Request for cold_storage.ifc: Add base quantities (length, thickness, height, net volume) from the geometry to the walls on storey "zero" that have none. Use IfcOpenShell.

First a look at what the model holds.

```python
import ifcopenshell
import ifcopenshell.util.element
import ifcopenshell.util.unit

model = ifcopenshell.open("cold_storage.ifc")
print(model.schema)
for unit_type in ("LENGTHUNIT", "AREAUNIT", "VOLUMEUNIT"):
    print(unit_type, ifcopenshell.util.unit.calculate_unit_scale(model, unit_type))
storey = next(s for s in model.by_type("IfcBuildingStorey") if s.Name == "zero")
walls = [e for e in ifcopenshell.util.element.get_decomposition(storey) if e.is_a("IfcWall")]
for e in sorted(walls, key=lambda e: e.id()):
    print(e.id(), e.is_a(), e.Name, list(ifcopenshell.util.element.get_psets(e, qtos_only=True)), sep=" | ")
```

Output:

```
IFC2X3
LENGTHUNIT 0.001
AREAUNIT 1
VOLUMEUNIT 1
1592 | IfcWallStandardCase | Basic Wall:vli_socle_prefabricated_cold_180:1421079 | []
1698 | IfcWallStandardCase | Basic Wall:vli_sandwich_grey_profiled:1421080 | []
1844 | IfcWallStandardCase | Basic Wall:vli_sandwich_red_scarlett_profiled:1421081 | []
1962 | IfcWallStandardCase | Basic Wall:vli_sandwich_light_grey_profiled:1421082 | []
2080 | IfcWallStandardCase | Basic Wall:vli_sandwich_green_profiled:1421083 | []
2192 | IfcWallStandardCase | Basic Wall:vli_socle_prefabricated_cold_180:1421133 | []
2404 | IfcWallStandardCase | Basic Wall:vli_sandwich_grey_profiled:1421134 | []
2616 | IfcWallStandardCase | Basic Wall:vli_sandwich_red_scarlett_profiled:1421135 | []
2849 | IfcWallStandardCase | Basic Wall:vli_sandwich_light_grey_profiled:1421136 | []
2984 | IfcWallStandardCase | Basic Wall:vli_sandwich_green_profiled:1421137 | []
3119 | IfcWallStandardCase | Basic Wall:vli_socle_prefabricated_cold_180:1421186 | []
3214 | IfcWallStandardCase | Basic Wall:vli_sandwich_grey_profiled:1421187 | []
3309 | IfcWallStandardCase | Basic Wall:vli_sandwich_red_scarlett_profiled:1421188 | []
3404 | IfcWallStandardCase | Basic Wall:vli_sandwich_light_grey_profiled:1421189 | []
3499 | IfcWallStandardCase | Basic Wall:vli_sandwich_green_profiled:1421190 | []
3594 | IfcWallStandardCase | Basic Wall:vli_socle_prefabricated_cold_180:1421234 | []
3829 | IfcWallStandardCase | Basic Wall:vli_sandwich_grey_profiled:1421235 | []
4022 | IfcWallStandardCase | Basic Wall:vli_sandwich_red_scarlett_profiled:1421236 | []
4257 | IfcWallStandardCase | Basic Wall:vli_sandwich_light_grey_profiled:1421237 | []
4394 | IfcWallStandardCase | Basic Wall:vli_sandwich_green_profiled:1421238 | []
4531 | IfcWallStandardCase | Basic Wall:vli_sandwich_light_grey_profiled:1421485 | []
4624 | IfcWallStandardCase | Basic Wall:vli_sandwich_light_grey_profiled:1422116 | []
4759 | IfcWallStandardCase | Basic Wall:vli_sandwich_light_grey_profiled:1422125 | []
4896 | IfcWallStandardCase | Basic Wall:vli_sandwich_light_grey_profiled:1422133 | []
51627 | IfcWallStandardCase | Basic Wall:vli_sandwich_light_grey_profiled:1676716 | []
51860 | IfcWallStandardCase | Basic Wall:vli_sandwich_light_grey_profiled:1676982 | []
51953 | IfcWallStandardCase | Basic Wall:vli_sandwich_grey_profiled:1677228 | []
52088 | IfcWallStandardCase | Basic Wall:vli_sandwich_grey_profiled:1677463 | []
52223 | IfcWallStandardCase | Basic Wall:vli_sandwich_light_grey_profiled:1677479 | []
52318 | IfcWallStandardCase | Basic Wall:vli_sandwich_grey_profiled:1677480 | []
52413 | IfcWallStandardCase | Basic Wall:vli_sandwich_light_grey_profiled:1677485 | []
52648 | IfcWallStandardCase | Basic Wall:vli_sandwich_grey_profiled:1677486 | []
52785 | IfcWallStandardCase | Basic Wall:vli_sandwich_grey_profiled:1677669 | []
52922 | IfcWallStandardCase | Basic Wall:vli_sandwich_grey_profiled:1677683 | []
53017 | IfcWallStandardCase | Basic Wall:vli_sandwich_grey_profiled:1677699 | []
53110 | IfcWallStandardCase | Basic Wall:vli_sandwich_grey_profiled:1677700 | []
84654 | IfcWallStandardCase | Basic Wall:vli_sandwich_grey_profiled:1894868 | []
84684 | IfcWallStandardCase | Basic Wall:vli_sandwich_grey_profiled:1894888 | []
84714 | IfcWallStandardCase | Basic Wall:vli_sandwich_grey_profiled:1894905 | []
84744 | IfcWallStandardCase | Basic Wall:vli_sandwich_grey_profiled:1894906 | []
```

```python
import ifcopenshell
import ifcopenshell.api.pset
import ifcopenshell.geom
import ifcopenshell.util.element
import ifcopenshell.util.shape
import ifcopenshell.util.unit

model = ifcopenshell.open("cold_storage.ifc")
unit_scale = ifcopenshell.util.unit.calculate_unit_scale(model)
volume_scale = ifcopenshell.util.unit.calculate_unit_scale(model, "VOLUMEUNIT")
settings = ifcopenshell.geom.settings()

storey = next(s for s in model.by_type("IfcBuildingStorey") if s.Name == "zero")
walls = [e for e in ifcopenshell.util.element.get_decomposition(storey) if e.is_a("IfcWall")]

for e in sorted(walls, key=lambda e: e.id()):
    if ifcopenshell.util.element.get_psets(e, qtos_only=True, should_inherit=False):
        continue
    # Geometry comes back in metres, in the element's own axes.
    shape = ifcopenshell.geom.create_shape(settings, e)
    values = {
        "Length": ifcopenshell.util.shape.get_x(shape.geometry) / unit_scale,
        "Width": ifcopenshell.util.shape.get_y(shape.geometry) / unit_scale,
        "Height": ifcopenshell.util.shape.get_z(shape.geometry) / unit_scale,
        "NetVolume": ifcopenshell.util.shape.get_volume(shape.geometry) / volume_scale,
    }
    qto = ifcopenshell.api.pset.add_qto(model, product=e, name="BaseQuantities")
    ifcopenshell.api.pset.edit_qto(model, qto=qto, properties=values)
    print(e.id(), {k: round(v, 3) for k, v in values.items()})

model.write("cold_storage_v2.ifc")
```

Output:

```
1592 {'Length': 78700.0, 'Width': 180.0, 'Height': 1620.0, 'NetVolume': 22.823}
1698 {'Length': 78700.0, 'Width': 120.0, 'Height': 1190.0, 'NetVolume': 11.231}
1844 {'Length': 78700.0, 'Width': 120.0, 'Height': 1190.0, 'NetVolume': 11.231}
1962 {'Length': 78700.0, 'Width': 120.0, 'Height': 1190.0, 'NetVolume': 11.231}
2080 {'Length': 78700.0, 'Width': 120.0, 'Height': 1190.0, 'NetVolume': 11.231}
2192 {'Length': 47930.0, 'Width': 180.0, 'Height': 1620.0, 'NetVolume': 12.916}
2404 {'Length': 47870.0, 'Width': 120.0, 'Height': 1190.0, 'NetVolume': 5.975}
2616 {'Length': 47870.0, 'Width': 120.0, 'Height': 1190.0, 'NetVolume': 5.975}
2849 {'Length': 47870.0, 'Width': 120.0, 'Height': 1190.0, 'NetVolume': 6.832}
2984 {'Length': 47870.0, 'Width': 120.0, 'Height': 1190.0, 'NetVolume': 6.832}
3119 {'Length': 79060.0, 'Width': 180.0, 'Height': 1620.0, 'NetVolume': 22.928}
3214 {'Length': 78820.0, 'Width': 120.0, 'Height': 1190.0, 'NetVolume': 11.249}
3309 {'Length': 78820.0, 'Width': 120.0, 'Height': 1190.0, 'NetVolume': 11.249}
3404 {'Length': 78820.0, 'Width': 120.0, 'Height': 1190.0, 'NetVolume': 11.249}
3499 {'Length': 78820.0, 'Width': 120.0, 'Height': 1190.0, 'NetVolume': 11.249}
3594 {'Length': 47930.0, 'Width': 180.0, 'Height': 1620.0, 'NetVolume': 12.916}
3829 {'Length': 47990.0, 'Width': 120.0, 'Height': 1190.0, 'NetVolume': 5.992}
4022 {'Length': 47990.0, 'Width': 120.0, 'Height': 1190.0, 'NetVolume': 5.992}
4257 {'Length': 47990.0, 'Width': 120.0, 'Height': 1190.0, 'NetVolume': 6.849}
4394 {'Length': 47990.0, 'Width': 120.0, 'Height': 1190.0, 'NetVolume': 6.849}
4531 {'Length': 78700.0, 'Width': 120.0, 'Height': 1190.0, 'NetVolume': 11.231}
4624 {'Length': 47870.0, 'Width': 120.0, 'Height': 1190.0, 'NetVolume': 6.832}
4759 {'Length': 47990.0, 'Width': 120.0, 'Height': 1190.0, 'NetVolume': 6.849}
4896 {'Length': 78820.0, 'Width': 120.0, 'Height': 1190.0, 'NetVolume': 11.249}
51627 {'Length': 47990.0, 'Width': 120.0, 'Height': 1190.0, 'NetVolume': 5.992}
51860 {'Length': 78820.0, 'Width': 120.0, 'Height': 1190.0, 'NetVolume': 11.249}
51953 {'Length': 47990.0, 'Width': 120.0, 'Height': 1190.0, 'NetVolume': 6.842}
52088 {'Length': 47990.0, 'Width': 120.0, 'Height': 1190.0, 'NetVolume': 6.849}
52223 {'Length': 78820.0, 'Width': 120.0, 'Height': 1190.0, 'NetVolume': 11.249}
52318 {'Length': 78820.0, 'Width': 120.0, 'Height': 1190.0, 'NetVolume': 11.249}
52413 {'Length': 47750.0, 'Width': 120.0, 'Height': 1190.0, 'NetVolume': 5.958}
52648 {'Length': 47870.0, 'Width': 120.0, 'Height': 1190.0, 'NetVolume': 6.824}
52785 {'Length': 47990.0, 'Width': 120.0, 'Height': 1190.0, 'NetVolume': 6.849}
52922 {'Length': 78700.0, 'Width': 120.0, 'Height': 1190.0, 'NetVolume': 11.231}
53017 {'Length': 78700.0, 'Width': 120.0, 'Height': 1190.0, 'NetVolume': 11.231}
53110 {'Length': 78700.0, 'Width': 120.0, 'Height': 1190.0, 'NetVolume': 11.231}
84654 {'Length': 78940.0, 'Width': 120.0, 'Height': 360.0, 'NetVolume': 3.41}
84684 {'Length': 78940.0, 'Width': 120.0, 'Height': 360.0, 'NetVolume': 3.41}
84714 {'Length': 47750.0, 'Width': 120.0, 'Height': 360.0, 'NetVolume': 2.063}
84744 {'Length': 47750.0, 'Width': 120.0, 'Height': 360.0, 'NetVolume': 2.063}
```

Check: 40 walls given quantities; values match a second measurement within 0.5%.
